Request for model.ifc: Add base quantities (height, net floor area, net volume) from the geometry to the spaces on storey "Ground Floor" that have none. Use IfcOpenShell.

First a look at what the model holds.

```python
import ifcopenshell
import ifcopenshell.util.element
import ifcopenshell.util.unit

model = ifcopenshell.open("model.ifc")
print(model.schema)
for unit_type in ("LENGTHUNIT", "AREAUNIT", "VOLUMEUNIT"):
    print(unit_type, ifcopenshell.util.unit.calculate_unit_scale(model, unit_type))
storey = next(s for s in model.by_type("IfcBuildingStorey") if s.Name == "Ground Floor")
spaces = [e for e in ifcopenshell.util.element.get_decomposition(storey) if e.is_a("IfcSpace")]
for e in sorted(spaces, key=lambda e: e.id()):
    print(e.id(), e.is_a(), e.Name, list(ifcopenshell.util.element.get_psets(e, qtos_only=True)), sep=" | ")
```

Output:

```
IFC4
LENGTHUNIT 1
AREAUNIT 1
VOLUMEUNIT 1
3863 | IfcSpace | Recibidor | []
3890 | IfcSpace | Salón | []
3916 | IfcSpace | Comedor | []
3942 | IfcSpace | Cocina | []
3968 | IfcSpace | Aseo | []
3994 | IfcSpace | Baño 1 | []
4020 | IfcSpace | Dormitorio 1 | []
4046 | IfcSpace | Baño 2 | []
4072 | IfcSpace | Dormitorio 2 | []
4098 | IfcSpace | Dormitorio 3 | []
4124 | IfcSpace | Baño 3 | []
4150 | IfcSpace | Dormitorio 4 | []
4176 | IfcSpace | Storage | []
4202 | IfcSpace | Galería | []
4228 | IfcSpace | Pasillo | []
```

```python
import ifcopenshell
import ifcopenshell.api.pset
import ifcopenshell.geom
import ifcopenshell.util.element
import ifcopenshell.util.shape
import ifcopenshell.util.unit

model = ifcopenshell.open("model.ifc")
unit_scale = ifcopenshell.util.unit.calculate_unit_scale(model)
area_scale = ifcopenshell.util.unit.calculate_unit_scale(model, "AREAUNIT")
volume_scale = ifcopenshell.util.unit.calculate_unit_scale(model, "VOLUMEUNIT")
settings = ifcopenshell.geom.settings()

storey = next(s for s in model.by_type("IfcBuildingStorey") if s.Name == "Ground Floor")
spaces = [e for e in ifcopenshell.util.element.get_decomposition(storey) if e.is_a("IfcSpace")]

for e in sorted(spaces, key=lambda e: e.id()):
    if ifcopenshell.util.element.get_psets(e, qtos_only=True, should_inherit=False):
        continue
    # Geometry comes back in metres, in the element's own axes.
    shape = ifcopenshell.geom.create_shape(settings, e)
    values = {
        "Height": ifcopenshell.util.shape.get_z(shape.geometry) / unit_scale,
        "NetFloorArea": ifcopenshell.util.shape.get_footprint_area(shape.geometry) / area_scale,
        "NetVolume": ifcopenshell.util.shape.get_volume(shape.geometry) / volume_scale,
    }
    qto = ifcopenshell.api.pset.add_qto(model, product=e, name="Qto_SpaceBaseQuantities")
    ifcopenshell.api.pset.edit_qto(model, qto=qto, properties=values)
    print(e.id(), {k: round(v, 3) for k, v in values.items()})

model.write("model_v2.ifc")
```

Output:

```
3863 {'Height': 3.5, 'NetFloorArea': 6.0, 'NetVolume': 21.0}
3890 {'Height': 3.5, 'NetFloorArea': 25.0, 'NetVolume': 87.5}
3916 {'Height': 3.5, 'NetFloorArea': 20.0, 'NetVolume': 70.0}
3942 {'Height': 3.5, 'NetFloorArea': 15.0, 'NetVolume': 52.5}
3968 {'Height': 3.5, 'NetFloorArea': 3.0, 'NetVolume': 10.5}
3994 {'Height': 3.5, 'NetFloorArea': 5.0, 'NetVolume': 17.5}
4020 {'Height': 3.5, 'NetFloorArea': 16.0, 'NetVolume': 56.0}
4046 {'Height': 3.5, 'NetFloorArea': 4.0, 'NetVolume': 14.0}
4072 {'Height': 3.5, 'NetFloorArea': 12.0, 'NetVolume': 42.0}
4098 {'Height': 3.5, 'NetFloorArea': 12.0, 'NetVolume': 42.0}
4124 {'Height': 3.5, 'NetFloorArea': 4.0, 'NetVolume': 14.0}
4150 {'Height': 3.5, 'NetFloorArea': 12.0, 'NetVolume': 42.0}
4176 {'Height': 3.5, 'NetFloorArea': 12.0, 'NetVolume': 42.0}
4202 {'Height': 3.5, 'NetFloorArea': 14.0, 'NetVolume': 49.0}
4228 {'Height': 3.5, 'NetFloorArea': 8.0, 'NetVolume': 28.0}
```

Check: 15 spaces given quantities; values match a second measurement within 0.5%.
